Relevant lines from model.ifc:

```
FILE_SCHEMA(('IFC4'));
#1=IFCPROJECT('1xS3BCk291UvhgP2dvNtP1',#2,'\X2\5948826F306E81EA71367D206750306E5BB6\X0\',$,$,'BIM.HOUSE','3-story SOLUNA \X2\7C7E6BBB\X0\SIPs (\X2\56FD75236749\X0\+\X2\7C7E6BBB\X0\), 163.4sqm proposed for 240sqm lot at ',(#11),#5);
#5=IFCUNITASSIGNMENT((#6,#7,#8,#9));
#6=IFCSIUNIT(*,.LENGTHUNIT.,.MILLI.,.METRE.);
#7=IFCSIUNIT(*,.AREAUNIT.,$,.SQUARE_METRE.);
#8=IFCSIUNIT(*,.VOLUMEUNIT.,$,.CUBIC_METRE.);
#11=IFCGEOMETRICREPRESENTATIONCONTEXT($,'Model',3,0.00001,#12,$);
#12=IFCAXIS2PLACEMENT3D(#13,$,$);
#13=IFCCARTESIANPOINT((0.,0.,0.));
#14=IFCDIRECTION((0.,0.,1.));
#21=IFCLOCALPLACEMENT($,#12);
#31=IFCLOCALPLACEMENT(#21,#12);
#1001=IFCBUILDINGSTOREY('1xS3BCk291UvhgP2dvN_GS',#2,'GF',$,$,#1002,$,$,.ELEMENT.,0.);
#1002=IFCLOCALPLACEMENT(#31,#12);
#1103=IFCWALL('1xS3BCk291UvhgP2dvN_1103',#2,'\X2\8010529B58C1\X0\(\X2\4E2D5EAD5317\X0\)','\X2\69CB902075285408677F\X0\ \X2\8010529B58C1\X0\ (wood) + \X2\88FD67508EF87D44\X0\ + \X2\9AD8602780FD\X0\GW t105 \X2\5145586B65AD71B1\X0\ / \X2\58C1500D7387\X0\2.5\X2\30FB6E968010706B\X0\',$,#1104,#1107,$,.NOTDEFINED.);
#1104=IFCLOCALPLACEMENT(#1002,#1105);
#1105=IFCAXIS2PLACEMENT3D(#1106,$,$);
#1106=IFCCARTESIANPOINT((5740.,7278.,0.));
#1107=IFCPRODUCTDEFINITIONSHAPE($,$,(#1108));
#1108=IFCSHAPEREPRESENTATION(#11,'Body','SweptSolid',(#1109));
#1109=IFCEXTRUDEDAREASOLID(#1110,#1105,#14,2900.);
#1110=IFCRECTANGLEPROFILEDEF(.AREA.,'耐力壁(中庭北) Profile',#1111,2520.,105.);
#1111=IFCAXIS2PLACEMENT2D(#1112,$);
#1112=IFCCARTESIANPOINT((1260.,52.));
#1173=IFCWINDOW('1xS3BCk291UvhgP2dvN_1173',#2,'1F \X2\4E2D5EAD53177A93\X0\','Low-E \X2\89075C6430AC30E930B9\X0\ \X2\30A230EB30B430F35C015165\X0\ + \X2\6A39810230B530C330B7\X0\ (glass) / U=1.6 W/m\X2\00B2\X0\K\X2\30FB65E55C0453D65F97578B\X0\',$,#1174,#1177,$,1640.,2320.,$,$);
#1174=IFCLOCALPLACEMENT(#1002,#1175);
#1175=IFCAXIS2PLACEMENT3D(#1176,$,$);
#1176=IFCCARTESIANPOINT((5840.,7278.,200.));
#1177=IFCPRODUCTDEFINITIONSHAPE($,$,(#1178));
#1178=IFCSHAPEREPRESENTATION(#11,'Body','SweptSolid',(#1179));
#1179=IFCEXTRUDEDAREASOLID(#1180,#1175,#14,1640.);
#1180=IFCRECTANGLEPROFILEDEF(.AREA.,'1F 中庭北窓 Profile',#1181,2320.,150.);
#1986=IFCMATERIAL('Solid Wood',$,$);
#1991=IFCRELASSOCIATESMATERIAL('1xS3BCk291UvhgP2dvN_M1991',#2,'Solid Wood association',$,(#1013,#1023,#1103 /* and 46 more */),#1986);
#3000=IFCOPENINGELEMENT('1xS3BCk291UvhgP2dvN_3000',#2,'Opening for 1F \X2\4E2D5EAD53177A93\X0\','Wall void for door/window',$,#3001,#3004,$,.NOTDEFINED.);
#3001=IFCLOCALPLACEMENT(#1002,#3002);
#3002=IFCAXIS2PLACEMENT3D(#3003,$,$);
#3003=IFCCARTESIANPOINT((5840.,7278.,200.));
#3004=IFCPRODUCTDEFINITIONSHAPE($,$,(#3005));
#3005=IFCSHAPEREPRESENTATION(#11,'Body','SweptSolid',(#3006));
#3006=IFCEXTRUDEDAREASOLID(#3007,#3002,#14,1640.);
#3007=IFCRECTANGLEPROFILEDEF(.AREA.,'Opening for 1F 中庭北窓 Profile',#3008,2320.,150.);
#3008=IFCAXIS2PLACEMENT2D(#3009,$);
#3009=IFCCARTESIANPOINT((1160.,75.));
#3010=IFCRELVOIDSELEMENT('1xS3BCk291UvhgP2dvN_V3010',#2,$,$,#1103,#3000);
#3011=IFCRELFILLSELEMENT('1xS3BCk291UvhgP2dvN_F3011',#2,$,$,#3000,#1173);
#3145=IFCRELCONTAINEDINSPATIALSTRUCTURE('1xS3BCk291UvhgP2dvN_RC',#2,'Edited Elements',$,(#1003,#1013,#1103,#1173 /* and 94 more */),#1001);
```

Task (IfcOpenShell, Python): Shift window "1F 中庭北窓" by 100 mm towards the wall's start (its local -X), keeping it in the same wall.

```python
import ifcopenshell
import ifcopenshell.api.geometry
import ifcopenshell.util.placement
import ifcopenshell.util.unit

model = ifcopenshell.open("model.ifc")
unit_scale = ifcopenshell.util.unit.calculate_unit_scale(model)

window = model.by_id(1173)
opening = window.FillsVoids[0].RelatingOpeningElement
wall = opening.VoidsElements[0].RelatingBuildingElement

wall_matrix = ifcopenshell.util.placement.get_local_placement(wall.ObjectPlacement)
shift = wall_matrix[:3, 0] * -0.1 / unit_scale
before = ifcopenshell.util.placement.get_local_placement(window.ObjectPlacement)[:3, 3].copy()

# The window is not placed relative to its opening, so move both.
for product in (opening, window):
    matrix = ifcopenshell.util.placement.get_local_placement(product.ObjectPlacement)
    matrix[:3, 3] += shift
    ifcopenshell.api.geometry.edit_object_placement(model, product=product, matrix=matrix, is_si=False)

after = ifcopenshell.util.placement.get_local_placement(window.ObjectPlacement)[:3, 3]
print("window moved by", (after - before).round(3) + 0.0)

model.write("model_updated.ifc")
```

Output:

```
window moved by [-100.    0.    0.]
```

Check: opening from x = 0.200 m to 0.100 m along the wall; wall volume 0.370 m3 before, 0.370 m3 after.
